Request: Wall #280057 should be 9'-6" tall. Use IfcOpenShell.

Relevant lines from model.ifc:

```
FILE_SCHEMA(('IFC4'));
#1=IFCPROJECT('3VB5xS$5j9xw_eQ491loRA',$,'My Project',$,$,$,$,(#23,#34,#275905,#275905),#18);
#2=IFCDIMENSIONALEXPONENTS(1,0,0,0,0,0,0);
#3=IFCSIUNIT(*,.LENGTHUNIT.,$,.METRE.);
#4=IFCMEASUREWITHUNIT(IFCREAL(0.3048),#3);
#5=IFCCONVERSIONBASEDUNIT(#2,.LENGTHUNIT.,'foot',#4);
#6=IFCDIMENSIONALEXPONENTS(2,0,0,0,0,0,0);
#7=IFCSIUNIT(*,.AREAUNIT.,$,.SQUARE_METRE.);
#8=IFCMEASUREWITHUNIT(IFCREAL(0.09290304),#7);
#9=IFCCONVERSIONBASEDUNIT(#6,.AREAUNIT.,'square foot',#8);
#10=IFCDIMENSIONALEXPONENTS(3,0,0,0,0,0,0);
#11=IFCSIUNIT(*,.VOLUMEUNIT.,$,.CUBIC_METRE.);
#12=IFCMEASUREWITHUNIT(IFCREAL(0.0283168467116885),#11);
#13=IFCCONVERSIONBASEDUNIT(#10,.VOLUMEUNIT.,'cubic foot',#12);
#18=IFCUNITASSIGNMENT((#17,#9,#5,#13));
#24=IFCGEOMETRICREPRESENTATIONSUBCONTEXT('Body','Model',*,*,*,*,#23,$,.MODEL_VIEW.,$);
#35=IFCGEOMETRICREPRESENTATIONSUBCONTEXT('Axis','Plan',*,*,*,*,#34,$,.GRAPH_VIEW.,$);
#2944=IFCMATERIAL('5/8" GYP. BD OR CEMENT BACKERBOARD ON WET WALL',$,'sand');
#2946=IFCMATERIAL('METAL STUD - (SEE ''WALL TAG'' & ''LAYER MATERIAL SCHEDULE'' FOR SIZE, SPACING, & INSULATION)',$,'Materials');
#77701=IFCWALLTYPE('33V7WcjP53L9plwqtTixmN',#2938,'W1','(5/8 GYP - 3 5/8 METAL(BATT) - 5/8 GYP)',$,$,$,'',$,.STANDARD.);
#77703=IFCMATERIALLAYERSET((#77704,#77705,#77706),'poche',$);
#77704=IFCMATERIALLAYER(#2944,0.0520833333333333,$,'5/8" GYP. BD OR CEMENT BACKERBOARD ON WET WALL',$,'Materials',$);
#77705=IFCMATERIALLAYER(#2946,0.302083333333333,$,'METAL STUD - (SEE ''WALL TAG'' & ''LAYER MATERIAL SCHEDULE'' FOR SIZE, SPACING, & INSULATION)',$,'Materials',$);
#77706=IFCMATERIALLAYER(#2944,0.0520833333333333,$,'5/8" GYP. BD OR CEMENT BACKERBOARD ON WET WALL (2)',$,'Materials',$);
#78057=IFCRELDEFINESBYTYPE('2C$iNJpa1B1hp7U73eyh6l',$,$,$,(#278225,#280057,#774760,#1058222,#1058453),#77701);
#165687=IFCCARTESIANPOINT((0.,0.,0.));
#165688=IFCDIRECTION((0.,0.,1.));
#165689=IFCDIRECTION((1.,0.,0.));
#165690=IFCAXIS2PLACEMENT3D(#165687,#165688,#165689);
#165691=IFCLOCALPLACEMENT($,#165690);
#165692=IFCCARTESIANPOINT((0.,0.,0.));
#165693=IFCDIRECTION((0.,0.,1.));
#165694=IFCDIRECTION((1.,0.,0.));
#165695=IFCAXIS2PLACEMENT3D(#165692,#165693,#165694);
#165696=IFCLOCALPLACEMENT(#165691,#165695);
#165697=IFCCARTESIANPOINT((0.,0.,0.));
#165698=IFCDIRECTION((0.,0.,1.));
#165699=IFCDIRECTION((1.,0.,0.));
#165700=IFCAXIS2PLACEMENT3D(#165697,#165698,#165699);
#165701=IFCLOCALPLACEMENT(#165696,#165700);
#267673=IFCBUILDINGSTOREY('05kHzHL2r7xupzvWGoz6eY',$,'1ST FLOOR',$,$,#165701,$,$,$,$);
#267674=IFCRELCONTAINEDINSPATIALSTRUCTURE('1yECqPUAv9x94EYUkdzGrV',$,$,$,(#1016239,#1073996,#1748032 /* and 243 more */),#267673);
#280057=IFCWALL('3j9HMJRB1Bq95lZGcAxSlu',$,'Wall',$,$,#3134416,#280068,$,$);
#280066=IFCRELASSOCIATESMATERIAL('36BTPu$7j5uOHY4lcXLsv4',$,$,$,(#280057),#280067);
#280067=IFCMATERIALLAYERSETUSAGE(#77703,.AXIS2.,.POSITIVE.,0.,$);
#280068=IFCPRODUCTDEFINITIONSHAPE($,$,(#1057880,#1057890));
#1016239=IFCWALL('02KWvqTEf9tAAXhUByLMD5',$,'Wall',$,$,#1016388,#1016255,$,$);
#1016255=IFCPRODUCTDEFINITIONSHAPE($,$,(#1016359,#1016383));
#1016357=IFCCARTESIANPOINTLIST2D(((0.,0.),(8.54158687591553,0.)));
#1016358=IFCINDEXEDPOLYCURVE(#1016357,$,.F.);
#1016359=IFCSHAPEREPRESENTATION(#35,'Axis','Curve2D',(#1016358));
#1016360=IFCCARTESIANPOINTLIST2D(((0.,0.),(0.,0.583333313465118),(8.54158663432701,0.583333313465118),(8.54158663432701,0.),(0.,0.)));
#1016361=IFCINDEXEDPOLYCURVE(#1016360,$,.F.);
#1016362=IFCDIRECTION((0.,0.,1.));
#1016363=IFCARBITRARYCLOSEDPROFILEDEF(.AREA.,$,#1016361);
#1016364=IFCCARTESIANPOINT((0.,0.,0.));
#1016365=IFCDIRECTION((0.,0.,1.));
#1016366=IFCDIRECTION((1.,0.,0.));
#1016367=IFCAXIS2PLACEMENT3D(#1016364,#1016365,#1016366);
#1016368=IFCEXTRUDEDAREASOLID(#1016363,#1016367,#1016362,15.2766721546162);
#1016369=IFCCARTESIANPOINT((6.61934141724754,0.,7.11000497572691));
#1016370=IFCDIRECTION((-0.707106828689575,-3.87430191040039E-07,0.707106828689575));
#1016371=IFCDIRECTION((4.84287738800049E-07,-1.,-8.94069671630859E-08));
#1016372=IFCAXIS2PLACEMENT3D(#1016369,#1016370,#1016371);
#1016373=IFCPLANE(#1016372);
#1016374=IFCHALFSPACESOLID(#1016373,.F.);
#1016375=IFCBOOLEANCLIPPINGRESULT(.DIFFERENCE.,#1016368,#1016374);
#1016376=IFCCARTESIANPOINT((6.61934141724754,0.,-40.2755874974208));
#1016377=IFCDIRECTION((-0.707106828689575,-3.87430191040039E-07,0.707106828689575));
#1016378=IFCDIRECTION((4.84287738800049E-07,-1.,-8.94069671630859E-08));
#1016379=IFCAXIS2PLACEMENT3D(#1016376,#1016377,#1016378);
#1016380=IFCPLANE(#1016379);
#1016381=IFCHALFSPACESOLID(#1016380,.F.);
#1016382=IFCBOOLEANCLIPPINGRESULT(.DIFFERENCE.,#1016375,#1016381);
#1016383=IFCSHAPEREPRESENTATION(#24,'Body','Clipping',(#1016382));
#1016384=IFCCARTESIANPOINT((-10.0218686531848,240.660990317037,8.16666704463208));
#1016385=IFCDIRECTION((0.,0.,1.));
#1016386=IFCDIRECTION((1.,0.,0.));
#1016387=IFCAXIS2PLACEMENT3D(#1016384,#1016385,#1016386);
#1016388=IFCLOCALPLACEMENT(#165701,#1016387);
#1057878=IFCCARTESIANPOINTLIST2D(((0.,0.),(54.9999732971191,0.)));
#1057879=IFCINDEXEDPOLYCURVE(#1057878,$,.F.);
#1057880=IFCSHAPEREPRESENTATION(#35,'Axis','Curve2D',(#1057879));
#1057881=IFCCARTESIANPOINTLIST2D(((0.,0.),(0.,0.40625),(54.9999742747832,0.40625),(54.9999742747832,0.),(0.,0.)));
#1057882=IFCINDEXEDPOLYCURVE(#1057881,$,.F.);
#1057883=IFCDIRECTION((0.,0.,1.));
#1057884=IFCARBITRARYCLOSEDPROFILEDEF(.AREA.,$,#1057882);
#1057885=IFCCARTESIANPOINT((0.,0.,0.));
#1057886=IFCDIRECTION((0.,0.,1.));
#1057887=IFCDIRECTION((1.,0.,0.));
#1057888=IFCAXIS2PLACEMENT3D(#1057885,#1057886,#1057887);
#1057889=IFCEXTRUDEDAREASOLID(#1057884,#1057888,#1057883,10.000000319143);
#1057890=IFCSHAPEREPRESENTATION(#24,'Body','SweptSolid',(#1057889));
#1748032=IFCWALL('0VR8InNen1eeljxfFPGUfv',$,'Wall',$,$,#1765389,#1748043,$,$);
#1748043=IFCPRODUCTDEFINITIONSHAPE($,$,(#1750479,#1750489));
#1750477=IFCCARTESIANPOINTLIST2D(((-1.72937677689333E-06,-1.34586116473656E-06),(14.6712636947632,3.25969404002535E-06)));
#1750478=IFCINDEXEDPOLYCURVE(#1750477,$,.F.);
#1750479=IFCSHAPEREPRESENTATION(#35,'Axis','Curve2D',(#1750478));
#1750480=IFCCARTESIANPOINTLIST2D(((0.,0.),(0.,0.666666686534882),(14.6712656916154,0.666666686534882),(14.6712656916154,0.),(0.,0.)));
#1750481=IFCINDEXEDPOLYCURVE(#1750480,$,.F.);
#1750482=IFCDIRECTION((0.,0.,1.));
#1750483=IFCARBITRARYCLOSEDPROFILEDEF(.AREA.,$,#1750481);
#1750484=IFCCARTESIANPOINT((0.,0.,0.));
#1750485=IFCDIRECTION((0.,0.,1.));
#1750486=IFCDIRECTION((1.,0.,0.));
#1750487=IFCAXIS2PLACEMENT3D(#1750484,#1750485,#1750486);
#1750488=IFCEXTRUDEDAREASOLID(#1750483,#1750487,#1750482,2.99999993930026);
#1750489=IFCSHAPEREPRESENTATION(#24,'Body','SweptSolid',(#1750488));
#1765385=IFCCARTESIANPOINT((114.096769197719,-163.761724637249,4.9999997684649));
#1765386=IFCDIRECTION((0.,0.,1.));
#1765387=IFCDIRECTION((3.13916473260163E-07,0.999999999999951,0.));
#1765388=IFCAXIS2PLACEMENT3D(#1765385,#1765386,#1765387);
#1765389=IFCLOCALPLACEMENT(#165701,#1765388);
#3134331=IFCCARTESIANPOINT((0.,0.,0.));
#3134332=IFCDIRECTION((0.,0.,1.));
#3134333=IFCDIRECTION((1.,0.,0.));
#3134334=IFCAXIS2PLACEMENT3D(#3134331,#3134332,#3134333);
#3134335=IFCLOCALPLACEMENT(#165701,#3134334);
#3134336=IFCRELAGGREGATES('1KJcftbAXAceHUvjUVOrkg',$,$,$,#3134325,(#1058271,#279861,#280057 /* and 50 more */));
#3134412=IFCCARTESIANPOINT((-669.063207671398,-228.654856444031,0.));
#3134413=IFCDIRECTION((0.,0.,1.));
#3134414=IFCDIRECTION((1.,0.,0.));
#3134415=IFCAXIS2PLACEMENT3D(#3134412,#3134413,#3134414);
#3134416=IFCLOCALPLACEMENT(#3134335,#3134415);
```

```python
import ifcopenshell
import ifcopenshell.geom
import ifcopenshell.util.representation
import ifcopenshell.util.shape
import ifcopenshell.util.unit

model = ifcopenshell.open("model.ifc")
unit_scale = ifcopenshell.util.unit.calculate_unit_scale(model)
settings = ifcopenshell.geom.settings()


def volume(element):
    """Net volume in cubic metres, openings subtracted."""
    shape = ifcopenshell.geom.create_shape(settings, element)
    return ifcopenshell.util.shape.get_volume(shape.geometry)


wall = model.by_id(280057)
before = volume(wall)

body = ifcopenshell.util.representation.get_representation(wall, "Model", "Body")
solid = body.Items[0]
old_height = solid.Depth
solid.Depth = 114 * 0.0254 / unit_scale
after = volume(wall)

print(f"height {old_height:g} -> {solid.Depth:g}, volume {before:.3f} -> {after:.3f} m3")

model.write("model_edited.ifc")
```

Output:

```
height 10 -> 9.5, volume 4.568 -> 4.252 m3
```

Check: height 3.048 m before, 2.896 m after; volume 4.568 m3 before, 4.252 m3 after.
